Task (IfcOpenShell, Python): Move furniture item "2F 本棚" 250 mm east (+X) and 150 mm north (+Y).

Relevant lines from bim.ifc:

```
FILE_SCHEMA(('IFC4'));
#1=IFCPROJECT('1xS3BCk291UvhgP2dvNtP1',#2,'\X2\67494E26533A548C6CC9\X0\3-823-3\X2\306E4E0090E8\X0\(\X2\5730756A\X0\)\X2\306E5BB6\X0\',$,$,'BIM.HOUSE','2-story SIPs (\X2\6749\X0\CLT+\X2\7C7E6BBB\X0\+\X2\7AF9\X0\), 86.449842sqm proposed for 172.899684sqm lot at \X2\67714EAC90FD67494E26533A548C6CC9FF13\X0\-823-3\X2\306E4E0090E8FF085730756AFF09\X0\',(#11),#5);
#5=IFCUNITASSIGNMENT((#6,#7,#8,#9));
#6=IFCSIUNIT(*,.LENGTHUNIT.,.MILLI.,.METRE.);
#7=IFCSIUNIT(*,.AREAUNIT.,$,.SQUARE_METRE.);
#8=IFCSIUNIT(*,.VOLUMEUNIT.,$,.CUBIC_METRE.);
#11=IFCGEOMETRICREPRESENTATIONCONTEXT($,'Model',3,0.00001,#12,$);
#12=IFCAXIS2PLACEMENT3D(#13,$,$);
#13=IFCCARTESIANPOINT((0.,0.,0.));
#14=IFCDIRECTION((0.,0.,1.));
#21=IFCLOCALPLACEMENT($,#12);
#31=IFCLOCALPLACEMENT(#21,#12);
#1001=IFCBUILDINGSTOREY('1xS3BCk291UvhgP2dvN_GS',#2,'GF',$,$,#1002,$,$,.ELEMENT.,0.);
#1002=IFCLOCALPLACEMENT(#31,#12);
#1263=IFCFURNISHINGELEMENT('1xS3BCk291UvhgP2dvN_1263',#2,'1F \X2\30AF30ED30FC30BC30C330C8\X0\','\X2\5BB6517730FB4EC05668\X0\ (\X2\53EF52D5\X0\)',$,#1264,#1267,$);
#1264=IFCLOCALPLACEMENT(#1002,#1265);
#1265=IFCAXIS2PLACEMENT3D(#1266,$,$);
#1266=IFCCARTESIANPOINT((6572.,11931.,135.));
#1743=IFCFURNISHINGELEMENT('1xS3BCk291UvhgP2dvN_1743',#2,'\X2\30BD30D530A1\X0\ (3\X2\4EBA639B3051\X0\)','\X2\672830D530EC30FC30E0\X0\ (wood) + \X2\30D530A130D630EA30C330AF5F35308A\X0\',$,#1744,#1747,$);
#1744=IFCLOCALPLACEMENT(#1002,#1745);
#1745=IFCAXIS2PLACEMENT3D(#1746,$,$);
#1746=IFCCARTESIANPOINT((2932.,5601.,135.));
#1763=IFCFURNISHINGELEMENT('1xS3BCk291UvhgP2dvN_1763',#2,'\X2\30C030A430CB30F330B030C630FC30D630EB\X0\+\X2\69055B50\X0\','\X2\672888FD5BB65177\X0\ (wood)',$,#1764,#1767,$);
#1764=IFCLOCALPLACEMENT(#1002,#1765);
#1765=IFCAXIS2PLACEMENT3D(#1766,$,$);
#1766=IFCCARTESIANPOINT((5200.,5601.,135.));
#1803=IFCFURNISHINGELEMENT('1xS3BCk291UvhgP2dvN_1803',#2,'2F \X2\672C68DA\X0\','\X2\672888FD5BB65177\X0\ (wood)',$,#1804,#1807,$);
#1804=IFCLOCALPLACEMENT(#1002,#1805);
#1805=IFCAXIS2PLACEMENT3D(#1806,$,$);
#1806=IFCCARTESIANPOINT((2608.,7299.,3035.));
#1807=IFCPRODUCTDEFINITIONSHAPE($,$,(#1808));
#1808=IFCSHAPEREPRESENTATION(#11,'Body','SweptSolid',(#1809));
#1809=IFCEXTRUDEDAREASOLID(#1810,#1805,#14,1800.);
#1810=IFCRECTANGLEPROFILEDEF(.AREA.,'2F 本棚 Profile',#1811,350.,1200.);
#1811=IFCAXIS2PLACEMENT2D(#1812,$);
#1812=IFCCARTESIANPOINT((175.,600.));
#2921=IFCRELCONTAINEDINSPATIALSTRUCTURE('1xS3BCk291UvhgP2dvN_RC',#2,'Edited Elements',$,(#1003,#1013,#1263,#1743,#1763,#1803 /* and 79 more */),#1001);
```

```python
import ifcopenshell
import ifcopenshell.api.geometry
import ifcopenshell.util.placement
import ifcopenshell.util.unit

model = ifcopenshell.open("bim.ifc")
unit_scale = ifcopenshell.util.unit.calculate_unit_scale(model)

item = model.by_guid("1xS3BCk291UvhgP2dvN_1803")
matrix = ifcopenshell.util.placement.get_local_placement(item.ObjectPlacement)
matrix[0, 3] += 0.25 / unit_scale
matrix[1, 3] += 0.15 / unit_scale
ifcopenshell.api.geometry.edit_object_placement(model, product=item, matrix=matrix, is_si=False)

print(ifcopenshell.util.placement.get_local_placement(item.ObjectPlacement).round(3) + 0.0)

model.write("bim_edited.ifc")
```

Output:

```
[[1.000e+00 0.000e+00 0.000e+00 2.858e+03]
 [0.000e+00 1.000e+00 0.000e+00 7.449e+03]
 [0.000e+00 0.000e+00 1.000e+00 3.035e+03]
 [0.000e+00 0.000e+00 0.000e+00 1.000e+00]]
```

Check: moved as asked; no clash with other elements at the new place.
